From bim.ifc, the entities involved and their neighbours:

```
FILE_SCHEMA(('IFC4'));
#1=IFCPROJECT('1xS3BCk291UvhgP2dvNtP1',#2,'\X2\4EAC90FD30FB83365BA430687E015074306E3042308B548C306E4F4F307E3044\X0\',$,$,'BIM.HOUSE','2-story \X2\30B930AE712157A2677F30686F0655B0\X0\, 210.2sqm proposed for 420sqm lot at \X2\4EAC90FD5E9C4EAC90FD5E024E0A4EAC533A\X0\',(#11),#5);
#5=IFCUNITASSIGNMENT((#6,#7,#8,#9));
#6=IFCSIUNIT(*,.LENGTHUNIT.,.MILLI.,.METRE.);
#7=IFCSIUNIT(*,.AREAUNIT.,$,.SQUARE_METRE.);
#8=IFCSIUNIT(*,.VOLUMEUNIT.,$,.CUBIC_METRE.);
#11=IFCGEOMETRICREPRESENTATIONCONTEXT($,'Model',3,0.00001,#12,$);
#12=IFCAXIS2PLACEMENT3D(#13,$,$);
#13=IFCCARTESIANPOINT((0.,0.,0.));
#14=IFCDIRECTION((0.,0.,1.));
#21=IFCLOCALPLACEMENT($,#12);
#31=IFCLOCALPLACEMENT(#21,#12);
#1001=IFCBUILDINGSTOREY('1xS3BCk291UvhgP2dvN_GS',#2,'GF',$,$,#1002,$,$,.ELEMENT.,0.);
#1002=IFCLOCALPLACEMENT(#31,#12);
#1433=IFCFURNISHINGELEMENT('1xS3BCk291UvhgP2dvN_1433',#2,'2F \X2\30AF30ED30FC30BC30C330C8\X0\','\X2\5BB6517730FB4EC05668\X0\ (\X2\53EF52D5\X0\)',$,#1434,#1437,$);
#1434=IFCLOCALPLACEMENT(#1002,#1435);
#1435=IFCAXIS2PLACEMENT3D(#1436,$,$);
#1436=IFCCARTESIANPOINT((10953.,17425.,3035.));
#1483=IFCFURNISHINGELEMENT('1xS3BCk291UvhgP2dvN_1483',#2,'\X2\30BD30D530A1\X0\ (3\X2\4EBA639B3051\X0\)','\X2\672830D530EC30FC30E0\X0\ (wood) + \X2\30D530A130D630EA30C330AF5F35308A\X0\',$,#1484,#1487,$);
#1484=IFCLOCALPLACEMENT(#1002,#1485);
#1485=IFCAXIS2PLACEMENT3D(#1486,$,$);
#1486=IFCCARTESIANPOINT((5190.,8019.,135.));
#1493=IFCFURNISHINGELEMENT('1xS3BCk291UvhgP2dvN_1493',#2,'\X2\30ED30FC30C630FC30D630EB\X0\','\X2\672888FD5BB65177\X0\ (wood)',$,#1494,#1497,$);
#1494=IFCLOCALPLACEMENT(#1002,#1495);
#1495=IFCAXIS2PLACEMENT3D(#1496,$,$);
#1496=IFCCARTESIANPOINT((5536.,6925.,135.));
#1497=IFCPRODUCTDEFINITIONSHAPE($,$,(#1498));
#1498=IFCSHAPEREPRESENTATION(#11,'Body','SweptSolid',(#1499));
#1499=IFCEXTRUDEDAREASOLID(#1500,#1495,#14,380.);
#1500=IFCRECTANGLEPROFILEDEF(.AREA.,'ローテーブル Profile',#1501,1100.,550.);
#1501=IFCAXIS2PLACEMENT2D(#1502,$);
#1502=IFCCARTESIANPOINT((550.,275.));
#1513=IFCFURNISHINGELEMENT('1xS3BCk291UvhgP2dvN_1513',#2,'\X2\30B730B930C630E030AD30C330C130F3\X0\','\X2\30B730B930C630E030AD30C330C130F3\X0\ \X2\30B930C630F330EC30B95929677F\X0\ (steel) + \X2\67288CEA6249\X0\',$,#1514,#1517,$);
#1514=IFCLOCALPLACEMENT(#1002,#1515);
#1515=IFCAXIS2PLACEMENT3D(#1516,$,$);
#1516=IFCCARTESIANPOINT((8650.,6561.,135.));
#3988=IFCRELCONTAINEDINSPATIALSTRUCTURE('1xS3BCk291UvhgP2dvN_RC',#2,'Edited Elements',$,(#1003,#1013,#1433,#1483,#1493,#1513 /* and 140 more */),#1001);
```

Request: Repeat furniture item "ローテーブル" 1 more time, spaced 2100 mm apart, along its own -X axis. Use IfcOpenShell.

```python
import ifcopenshell
import ifcopenshell.api.geometry
import ifcopenshell.api.root
import ifcopenshell.util.element
import ifcopenshell.util.placement

model = ifcopenshell.open("bim.ifc")


def reuse_history(source, copy):
    """copy_class also copies each property set's owner history, people and application; keep the originals."""
    for rel in copy.IsDefinedBy:
        if rel.is_a("IfcRelDefinesByProperties") and (history := rel.RelatingPropertyDefinition.OwnerHistory):
            rel.RelatingPropertyDefinition.OwnerHistory = source.OwnerHistory
            ifcopenshell.util.element.remove_deep2(model, history)


source = model.by_guid("1xS3BCk291UvhgP2dvN_1493")
base = ifcopenshell.util.placement.get_local_placement(source.ObjectPlacement)
step = -base[:3, 0] * 2100.0

for i in range(1, 2):
    copy = ifcopenshell.api.root.copy_class(model, product=source)
    copy.Representation = ifcopenshell.util.element.copy_deep(
        model, source.Representation, exclude=["IfcGeometricRepresentationContext", "IfcRepresentationMap"]
    )
    reuse_history(source, copy)
    matrix = base.copy()
    matrix[:3, 3] += i * step
    print("added at", matrix[:3, 3].round(3) + 0.0)
    ifcopenshell.api.geometry.edit_object_placement(model, product=copy, matrix=matrix, is_si=False)

model.write("bim_edited.ifc")
```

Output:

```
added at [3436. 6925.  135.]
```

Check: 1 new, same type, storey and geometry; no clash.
